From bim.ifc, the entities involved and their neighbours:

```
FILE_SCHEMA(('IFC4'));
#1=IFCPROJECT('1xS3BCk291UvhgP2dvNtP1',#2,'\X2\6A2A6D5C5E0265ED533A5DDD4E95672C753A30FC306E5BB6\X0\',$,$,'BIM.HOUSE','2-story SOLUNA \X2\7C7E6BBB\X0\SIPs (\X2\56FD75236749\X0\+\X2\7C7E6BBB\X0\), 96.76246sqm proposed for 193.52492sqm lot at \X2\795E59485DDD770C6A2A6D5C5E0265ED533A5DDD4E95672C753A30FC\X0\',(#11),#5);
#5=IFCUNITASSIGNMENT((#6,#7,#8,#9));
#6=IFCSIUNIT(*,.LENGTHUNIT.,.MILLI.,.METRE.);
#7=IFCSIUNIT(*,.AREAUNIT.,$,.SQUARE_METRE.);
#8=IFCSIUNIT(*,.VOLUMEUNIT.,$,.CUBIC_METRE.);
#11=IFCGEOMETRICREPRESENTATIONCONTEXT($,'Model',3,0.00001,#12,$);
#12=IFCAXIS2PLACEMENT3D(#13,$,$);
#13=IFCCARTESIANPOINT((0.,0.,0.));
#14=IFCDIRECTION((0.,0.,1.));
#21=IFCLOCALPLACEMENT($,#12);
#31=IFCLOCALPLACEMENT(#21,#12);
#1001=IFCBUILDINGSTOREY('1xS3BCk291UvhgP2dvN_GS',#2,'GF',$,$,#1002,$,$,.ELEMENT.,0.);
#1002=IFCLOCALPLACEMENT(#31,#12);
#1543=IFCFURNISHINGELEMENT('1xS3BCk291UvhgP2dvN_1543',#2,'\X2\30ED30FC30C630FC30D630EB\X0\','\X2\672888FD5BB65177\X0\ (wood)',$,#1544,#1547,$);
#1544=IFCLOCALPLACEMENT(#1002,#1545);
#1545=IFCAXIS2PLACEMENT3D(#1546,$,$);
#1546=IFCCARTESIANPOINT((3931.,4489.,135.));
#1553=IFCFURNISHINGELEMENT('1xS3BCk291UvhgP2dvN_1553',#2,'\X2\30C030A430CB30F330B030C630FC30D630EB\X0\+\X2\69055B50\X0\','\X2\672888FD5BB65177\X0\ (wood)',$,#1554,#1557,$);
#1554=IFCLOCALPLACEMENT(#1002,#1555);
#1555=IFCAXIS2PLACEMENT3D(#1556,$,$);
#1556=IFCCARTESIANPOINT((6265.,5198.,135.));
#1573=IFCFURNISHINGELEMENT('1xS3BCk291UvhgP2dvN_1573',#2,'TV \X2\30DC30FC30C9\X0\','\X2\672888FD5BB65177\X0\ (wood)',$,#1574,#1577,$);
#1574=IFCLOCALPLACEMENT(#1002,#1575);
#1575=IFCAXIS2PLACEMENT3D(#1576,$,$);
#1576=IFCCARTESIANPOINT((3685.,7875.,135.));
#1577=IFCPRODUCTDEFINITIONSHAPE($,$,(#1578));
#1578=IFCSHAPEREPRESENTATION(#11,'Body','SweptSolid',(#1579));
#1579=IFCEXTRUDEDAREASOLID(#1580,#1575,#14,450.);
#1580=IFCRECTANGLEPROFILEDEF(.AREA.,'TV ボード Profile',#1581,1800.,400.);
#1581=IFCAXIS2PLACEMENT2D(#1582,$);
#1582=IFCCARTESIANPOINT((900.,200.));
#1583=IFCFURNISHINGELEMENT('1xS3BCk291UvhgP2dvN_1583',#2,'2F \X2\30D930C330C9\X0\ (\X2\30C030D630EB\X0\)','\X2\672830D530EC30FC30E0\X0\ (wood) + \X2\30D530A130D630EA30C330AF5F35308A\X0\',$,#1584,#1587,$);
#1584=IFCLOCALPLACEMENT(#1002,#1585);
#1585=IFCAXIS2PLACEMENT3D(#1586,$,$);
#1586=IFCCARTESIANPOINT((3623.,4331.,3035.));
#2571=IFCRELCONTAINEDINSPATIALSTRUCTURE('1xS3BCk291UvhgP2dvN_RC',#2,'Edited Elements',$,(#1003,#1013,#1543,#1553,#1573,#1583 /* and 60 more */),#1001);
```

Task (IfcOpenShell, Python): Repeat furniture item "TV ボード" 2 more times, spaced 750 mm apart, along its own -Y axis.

```python
import ifcopenshell
import ifcopenshell.api.geometry
import ifcopenshell.api.root
import ifcopenshell.util.element
import ifcopenshell.util.placement

model = ifcopenshell.open("bim.ifc")


def reuse_history(source, copy):
    """copy_class also copies each property set's owner history, people and application; keep the originals."""
    for rel in copy.IsDefinedBy:
        if rel.is_a("IfcRelDefinesByProperties") and (history := rel.RelatingPropertyDefinition.OwnerHistory):
            rel.RelatingPropertyDefinition.OwnerHistory = source.OwnerHistory
            ifcopenshell.util.element.remove_deep2(model, history)


source = model.by_guid("1xS3BCk291UvhgP2dvN_1573")
base = ifcopenshell.util.placement.get_local_placement(source.ObjectPlacement)
step = -base[:3, 1] * 750.0

for i in range(1, 3):
    copy = ifcopenshell.api.root.copy_class(model, product=source)
    copy.Representation = ifcopenshell.util.element.copy_deep(
        model, source.Representation, exclude=["IfcGeometricRepresentationContext", "IfcRepresentationMap"]
    )
    reuse_history(source, copy)
    matrix = base.copy()
    matrix[:3, 3] += i * step
    print("added at", matrix[:3, 3].round(3) + 0.0)
    ifcopenshell.api.geometry.edit_object_placement(model, product=copy, matrix=matrix, is_si=False)

model.write("bim_rev.ifc")
```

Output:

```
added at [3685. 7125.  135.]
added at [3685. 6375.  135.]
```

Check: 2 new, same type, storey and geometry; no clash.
